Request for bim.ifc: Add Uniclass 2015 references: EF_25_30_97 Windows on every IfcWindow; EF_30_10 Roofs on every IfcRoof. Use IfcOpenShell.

First a look at what the model holds.

```python
import ifcopenshell

model = ifcopenshell.open("bim.ifc")
print(model.schema)
print("classifications:", [c.Name for c in model.by_type("IfcClassification")])
for ifc_class in ("IfcDoor", "IfcRoof", "IfcStair", "IfcWall", "IfcWindow"):
    print(ifc_class, len(model.by_type(ifc_class)))
```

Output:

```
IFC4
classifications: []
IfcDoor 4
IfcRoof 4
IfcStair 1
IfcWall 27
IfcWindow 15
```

```python
import ifcopenshell
import ifcopenshell.api.classification

model = ifcopenshell.open("bim.ifc")

system = ifcopenshell.api.classification.add_classification(model, classification="Uniclass 2015")

codes = {
    "IfcWindow": ("EF_25_30_97", "Windows"),
    "IfcRoof": ("EF_30_10", "Roofs"),
}
for ifc_class, (code, name) in codes.items():
    products = model.by_type(ifc_class)
    ifcopenshell.api.classification.add_reference(
        model, products=products, classification=system, identification=code, name=name
    )
    print(code, len(products))

model.write("bim_updated.ifc")
```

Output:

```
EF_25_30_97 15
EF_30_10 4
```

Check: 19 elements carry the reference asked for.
